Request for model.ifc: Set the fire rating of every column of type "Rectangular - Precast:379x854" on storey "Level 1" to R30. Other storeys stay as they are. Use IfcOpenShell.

First a look at what the model holds.

```python
import ifcopenshell
import ifcopenshell.util.element

model = ifcopenshell.open("model.ifc")
print(model.schema)
storey = next(s for s in model.by_type("IfcBuildingStorey") if s.Name == "Level 1")
columns = [e for e in ifcopenshell.util.element.get_decomposition(storey) if e.is_a("IfcColumn")]
seen = {}
for e in columns:
    element_type = ifcopenshell.util.element.get_type(e)
    key = (element_type.Name if element_type != e and element_type else None, ifcopenshell.util.element.get_pset(e, "Pset_ColumnCommon", "FireRating"))
    seen[key] = seen.get(key, 0) + 1
for (name, value), count in sorted(seen.items(), key=str):
    print(count, "x", name, "|", value)
```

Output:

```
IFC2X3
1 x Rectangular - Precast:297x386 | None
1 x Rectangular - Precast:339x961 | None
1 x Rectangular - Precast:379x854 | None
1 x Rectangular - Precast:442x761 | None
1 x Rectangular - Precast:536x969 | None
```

```python
import ifcopenshell
import ifcopenshell.api.pset
import ifcopenshell.util.element

model = ifcopenshell.open("model.ifc")

storey = next(s for s in model.by_type("IfcBuildingStorey") if s.Name == "Level 1")
columns = [e for e in ifcopenshell.util.element.get_decomposition(storey) if e.is_a("IfcColumn")]

count = 0
for e in columns:
    element_type = ifcopenshell.util.element.get_type(e)
    if element_type in (None, e) or element_type.Name != "Rectangular - Precast:379x854":
        continue
    # add_pset returns the element's existing set when there is one.
    pset = ifcopenshell.api.pset.add_pset(model, product=e, name="Pset_ColumnCommon")
    ifcopenshell.api.pset.edit_pset(model, pset=pset, properties={"FireRating": "R30"})
    count += 1

print(count, "columns updated")

model.write("model-out.ifc")
```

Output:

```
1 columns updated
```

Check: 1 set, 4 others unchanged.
